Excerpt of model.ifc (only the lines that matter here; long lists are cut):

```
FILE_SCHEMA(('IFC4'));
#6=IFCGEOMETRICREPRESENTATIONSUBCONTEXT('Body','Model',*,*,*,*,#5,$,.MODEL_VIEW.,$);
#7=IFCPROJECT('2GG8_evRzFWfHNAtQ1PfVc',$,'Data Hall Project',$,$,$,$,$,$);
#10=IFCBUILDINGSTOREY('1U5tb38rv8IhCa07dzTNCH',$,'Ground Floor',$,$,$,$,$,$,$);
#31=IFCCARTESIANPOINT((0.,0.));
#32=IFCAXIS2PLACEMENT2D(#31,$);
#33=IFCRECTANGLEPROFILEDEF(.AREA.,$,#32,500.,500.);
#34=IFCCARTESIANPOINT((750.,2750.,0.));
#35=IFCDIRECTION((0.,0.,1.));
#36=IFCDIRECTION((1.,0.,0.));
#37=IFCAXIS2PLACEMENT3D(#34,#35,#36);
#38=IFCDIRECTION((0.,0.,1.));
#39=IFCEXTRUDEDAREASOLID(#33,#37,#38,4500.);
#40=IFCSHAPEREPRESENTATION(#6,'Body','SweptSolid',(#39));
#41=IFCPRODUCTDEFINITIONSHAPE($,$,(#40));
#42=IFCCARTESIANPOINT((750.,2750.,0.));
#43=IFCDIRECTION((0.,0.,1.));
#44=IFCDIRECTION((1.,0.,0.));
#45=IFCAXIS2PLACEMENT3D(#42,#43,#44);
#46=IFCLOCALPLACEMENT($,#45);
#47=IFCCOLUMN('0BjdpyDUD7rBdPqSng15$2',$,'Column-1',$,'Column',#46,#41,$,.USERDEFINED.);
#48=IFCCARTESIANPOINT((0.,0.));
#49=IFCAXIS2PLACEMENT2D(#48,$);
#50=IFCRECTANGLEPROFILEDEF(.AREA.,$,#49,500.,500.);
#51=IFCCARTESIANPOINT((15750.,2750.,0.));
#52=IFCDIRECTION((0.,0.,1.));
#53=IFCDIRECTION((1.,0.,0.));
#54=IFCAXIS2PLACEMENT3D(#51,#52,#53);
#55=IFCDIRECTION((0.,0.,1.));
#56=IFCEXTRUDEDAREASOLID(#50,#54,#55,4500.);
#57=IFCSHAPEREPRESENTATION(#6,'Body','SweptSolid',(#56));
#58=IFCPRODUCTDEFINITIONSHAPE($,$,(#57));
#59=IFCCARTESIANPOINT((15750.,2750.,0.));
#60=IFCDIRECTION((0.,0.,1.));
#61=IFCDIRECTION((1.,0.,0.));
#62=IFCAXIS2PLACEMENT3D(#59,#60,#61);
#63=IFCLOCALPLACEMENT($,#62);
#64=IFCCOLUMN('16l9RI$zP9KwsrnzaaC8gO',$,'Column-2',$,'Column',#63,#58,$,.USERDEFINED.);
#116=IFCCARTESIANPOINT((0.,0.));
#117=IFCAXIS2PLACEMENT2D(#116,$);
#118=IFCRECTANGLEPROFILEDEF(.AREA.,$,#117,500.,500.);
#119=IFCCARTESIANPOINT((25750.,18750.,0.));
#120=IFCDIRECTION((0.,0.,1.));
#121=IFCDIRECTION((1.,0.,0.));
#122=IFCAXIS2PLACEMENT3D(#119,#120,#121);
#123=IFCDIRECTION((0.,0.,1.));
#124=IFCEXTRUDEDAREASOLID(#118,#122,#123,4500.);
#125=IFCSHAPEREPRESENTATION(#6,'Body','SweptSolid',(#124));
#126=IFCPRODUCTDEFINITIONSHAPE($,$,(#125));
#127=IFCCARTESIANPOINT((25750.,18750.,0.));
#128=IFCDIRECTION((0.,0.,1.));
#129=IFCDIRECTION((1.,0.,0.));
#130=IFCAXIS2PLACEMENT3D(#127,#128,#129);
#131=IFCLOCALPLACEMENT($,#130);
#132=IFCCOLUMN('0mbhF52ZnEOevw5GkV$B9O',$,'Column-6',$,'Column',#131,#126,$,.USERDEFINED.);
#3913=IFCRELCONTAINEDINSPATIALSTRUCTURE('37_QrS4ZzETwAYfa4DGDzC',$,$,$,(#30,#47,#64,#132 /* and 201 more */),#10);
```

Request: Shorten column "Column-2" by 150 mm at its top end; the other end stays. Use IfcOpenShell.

```python
import ifcopenshell
import ifcopenshell.util.representation
import ifcopenshell.util.unit

model = ifcopenshell.open("model.ifc")
unit_scale = ifcopenshell.util.unit.calculate_unit_scale(model)

member = model.by_guid("16l9RI$zP9KwsrnzaaC8gO")
change = -0.15 / unit_scale

# The extrusion runs towards the end named, so only its depth changes.
body = ifcopenshell.util.representation.get_representation(member, "Model", "Body")
solid = body.Items[0]
old_length = solid.Depth
solid.Depth += change

print(f"length {old_length:g} -> {solid.Depth:g}")

model.write("model_updated.ifc")
```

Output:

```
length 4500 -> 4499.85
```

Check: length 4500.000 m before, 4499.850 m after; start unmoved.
